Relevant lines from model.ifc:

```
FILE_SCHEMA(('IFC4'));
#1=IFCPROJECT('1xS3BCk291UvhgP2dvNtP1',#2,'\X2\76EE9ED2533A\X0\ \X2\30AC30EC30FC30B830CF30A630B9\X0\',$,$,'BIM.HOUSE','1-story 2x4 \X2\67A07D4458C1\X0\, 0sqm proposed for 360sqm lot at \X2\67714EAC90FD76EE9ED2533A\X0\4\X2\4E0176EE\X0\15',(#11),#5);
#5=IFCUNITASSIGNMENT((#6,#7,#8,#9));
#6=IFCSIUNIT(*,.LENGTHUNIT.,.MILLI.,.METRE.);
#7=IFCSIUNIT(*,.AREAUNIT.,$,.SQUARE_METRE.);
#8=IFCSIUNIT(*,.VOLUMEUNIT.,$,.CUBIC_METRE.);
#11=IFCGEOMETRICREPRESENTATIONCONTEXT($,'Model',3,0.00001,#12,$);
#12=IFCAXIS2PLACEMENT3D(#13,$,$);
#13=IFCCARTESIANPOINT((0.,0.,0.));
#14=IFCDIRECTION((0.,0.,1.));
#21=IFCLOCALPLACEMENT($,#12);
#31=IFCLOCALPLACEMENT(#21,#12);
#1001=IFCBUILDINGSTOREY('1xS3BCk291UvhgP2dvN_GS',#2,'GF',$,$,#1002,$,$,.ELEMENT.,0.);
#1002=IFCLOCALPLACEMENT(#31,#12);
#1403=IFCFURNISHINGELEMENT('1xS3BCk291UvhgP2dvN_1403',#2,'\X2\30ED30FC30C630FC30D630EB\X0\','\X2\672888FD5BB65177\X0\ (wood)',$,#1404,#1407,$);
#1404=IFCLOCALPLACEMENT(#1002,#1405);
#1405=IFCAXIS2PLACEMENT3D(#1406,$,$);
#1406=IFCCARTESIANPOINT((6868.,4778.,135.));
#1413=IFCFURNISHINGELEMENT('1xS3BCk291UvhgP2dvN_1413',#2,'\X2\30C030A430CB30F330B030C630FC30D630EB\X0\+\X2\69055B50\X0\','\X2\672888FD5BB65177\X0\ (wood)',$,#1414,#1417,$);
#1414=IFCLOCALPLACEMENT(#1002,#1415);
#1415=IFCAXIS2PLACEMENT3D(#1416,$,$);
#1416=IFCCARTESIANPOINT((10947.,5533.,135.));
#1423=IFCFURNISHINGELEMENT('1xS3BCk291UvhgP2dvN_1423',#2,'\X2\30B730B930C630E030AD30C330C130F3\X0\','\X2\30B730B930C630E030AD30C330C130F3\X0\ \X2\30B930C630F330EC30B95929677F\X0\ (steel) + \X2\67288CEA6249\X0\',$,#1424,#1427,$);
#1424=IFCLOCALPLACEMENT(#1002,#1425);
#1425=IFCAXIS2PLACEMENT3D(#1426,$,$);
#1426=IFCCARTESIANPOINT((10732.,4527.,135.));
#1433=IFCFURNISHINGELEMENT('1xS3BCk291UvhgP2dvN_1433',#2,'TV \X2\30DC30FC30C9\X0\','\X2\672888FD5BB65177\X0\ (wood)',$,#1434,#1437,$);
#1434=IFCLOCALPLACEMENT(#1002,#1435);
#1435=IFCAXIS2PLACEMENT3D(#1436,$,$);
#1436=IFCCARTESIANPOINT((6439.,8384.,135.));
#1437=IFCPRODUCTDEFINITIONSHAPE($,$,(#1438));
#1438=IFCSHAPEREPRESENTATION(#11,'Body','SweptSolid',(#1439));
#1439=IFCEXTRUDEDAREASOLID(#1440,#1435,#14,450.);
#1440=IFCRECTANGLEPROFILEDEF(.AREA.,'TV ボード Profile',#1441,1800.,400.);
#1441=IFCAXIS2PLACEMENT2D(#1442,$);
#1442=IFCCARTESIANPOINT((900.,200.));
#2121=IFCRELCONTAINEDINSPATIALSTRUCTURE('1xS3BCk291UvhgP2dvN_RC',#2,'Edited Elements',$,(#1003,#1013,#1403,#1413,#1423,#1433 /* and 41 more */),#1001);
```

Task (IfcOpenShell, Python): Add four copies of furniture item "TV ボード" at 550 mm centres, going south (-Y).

```python
import numpy as np
import ifcopenshell
import ifcopenshell.api.geometry
import ifcopenshell.api.root
import ifcopenshell.util.element
import ifcopenshell.util.placement

model = ifcopenshell.open("model.ifc")


def reuse_history(source, copy):
    """copy_class also copies each property set's owner history, people and application; keep the originals."""
    for rel in copy.IsDefinedBy:
        if rel.is_a("IfcRelDefinesByProperties") and (history := rel.RelatingPropertyDefinition.OwnerHistory):
            rel.RelatingPropertyDefinition.OwnerHistory = source.OwnerHistory
            ifcopenshell.util.element.remove_deep2(model, history)


source = model.by_id(1433)
base = ifcopenshell.util.placement.get_local_placement(source.ObjectPlacement)
step = np.array([0.0, -1.0, 0.0]) * 550.0

for i in range(1, 5):
    copy = ifcopenshell.api.root.copy_class(model, product=source)
    copy.Representation = ifcopenshell.util.element.copy_deep(
        model, source.Representation, exclude=["IfcGeometricRepresentationContext", "IfcRepresentationMap"]
    )
    reuse_history(source, copy)
    matrix = base.copy()
    matrix[:3, 3] += i * step
    print("added at", matrix[:3, 3].round(3) + 0.0)
    ifcopenshell.api.geometry.edit_object_placement(model, product=copy, matrix=matrix, is_si=False)

model.write("model_rev.ifc")
```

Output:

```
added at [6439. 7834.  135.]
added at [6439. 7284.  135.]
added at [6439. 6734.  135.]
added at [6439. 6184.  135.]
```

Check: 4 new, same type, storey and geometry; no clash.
